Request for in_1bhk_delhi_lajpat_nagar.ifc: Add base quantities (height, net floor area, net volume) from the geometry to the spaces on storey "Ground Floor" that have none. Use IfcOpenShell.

First a look at what the model holds.

```python
import ifcopenshell
import ifcopenshell.util.element
import ifcopenshell.util.unit

model = ifcopenshell.open("in_1bhk_delhi_lajpat_nagar.ifc")
print(model.schema)
for unit_type in ("LENGTHUNIT", "AREAUNIT", "VOLUMEUNIT"):
    print(unit_type, ifcopenshell.util.unit.calculate_unit_scale(model, unit_type))
storey = next(s for s in model.by_type("IfcBuildingStorey") if s.Name == "Ground Floor")
spaces = [e for e in ifcopenshell.util.element.get_decomposition(storey) if e.is_a("IfcSpace")]
for e in sorted(spaces, key=lambda e: e.id()):
    print(e.id(), e.is_a(), e.Name, list(ifcopenshell.util.element.get_psets(e, qtos_only=True)), sep=" | ")
```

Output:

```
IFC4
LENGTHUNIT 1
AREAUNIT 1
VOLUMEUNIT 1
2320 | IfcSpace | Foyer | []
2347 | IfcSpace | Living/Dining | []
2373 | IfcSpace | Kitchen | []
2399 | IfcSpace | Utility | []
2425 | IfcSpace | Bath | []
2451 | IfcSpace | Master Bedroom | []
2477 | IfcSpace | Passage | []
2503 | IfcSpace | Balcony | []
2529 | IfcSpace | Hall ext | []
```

```python
import ifcopenshell
import ifcopenshell.api.pset
import ifcopenshell.geom
import ifcopenshell.util.element
import ifcopenshell.util.shape
import ifcopenshell.util.unit

model = ifcopenshell.open("in_1bhk_delhi_lajpat_nagar.ifc")
unit_scale = ifcopenshell.util.unit.calculate_unit_scale(model)
area_scale = ifcopenshell.util.unit.calculate_unit_scale(model, "AREAUNIT")
volume_scale = ifcopenshell.util.unit.calculate_unit_scale(model, "VOLUMEUNIT")
settings = ifcopenshell.geom.settings()

storey = next(s for s in model.by_type("IfcBuildingStorey") if s.Name == "Ground Floor")
spaces = [e for e in ifcopenshell.util.element.get_decomposition(storey) if e.is_a("IfcSpace")]

for e in sorted(spaces, key=lambda e: e.id()):
    if ifcopenshell.util.element.get_psets(e, qtos_only=True, should_inherit=False):
        continue
    # Geometry comes back in metres, in the element's own axes.
    shape = ifcopenshell.geom.create_shape(settings, e)
    values = {
        "Height": ifcopenshell.util.shape.get_z(shape.geometry) / unit_scale,
        "NetFloorArea": ifcopenshell.util.shape.get_footprint_area(shape.geometry) / area_scale,
        "NetVolume": ifcopenshell.util.shape.get_volume(shape.geometry) / volume_scale,
    }
    qto = ifcopenshell.api.pset.add_qto(model, product=e, name="Qto_SpaceBaseQuantities")
    ifcopenshell.api.pset.edit_qto(model, qto=qto, properties=values)
    print(e.id(), {k: round(v, 3) for k, v in values.items()})

model.write("in_1bhk_delhi_lajpat_nagar_v2.ifc")
```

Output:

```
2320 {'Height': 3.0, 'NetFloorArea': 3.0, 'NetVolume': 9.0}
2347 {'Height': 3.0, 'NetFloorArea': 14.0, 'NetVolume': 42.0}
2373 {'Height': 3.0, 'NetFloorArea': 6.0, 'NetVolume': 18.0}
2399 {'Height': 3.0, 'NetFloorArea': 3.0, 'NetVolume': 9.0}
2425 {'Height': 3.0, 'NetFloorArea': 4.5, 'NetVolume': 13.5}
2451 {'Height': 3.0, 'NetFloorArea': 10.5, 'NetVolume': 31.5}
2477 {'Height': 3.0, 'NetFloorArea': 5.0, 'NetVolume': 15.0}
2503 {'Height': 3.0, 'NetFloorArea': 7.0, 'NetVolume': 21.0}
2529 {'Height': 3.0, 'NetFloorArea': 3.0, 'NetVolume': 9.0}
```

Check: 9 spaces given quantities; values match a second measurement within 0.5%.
